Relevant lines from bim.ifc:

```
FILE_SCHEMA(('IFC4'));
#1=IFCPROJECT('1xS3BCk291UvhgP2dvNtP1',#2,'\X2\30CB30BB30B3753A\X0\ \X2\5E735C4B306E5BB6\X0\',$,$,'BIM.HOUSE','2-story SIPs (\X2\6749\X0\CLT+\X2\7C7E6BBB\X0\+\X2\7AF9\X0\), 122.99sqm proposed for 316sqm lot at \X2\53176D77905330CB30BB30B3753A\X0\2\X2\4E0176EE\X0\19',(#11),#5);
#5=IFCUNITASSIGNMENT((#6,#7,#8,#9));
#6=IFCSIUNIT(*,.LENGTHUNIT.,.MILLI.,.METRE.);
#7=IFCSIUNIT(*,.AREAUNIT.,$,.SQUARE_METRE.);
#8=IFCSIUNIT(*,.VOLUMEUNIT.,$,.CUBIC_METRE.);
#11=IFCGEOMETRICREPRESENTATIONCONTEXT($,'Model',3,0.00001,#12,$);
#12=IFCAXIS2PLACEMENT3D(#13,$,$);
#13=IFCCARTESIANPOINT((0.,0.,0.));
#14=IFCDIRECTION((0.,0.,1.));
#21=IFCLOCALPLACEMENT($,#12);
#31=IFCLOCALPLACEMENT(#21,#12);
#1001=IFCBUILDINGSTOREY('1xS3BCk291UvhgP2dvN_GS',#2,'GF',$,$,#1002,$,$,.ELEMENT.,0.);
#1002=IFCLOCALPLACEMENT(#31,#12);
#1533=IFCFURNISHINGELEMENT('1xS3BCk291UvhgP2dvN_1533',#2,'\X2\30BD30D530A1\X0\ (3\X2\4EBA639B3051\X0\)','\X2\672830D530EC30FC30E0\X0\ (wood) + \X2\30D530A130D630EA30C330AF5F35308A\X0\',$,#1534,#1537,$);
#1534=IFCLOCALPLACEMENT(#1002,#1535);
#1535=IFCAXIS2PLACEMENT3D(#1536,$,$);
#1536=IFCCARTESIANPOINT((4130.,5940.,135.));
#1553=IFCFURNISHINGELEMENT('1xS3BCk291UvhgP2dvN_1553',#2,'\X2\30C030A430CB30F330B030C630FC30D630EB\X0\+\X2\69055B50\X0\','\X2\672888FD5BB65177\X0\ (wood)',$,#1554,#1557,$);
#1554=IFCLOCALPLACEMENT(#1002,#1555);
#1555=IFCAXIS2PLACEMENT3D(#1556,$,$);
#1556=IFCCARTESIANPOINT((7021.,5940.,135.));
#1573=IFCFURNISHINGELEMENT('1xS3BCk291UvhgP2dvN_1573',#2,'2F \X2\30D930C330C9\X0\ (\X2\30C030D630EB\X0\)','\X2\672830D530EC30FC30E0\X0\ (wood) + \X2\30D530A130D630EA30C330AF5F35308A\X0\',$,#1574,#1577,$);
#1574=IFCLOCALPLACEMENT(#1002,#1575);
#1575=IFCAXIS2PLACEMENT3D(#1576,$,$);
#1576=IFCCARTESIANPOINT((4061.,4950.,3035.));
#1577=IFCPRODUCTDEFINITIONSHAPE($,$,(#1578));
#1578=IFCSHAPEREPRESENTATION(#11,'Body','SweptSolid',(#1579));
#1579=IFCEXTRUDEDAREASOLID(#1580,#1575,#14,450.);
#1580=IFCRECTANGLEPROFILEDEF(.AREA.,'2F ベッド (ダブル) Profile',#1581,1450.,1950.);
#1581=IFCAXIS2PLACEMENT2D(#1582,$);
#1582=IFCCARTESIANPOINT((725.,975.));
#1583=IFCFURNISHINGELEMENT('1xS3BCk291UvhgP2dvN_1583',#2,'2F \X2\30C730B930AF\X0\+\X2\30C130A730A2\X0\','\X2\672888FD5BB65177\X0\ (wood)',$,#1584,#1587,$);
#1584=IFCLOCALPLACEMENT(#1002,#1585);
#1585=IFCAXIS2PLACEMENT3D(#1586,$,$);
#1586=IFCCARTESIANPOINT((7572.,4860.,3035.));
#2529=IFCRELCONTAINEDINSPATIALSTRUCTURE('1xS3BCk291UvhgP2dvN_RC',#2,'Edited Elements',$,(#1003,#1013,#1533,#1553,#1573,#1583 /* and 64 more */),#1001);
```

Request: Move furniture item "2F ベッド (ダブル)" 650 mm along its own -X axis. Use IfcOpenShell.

```python
import ifcopenshell
import ifcopenshell.api.geometry
import ifcopenshell.util.placement

model = ifcopenshell.open("bim.ifc")

item = model.by_guid("1xS3BCk291UvhgP2dvN_1573")
matrix = ifcopenshell.util.placement.get_local_placement(item.ObjectPlacement)
matrix[:3, 3] -= matrix[:3, 0] * 650.0
ifcopenshell.api.geometry.edit_object_placement(model, product=item, matrix=matrix, is_si=False)

print(ifcopenshell.util.placement.get_local_placement(item.ObjectPlacement).round(3) + 0.0)

model.write("bim_edited.ifc")
```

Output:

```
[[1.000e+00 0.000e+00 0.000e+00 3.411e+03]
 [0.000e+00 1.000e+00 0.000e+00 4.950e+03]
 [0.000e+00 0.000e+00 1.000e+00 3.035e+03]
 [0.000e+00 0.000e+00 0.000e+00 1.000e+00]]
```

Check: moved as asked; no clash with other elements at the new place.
